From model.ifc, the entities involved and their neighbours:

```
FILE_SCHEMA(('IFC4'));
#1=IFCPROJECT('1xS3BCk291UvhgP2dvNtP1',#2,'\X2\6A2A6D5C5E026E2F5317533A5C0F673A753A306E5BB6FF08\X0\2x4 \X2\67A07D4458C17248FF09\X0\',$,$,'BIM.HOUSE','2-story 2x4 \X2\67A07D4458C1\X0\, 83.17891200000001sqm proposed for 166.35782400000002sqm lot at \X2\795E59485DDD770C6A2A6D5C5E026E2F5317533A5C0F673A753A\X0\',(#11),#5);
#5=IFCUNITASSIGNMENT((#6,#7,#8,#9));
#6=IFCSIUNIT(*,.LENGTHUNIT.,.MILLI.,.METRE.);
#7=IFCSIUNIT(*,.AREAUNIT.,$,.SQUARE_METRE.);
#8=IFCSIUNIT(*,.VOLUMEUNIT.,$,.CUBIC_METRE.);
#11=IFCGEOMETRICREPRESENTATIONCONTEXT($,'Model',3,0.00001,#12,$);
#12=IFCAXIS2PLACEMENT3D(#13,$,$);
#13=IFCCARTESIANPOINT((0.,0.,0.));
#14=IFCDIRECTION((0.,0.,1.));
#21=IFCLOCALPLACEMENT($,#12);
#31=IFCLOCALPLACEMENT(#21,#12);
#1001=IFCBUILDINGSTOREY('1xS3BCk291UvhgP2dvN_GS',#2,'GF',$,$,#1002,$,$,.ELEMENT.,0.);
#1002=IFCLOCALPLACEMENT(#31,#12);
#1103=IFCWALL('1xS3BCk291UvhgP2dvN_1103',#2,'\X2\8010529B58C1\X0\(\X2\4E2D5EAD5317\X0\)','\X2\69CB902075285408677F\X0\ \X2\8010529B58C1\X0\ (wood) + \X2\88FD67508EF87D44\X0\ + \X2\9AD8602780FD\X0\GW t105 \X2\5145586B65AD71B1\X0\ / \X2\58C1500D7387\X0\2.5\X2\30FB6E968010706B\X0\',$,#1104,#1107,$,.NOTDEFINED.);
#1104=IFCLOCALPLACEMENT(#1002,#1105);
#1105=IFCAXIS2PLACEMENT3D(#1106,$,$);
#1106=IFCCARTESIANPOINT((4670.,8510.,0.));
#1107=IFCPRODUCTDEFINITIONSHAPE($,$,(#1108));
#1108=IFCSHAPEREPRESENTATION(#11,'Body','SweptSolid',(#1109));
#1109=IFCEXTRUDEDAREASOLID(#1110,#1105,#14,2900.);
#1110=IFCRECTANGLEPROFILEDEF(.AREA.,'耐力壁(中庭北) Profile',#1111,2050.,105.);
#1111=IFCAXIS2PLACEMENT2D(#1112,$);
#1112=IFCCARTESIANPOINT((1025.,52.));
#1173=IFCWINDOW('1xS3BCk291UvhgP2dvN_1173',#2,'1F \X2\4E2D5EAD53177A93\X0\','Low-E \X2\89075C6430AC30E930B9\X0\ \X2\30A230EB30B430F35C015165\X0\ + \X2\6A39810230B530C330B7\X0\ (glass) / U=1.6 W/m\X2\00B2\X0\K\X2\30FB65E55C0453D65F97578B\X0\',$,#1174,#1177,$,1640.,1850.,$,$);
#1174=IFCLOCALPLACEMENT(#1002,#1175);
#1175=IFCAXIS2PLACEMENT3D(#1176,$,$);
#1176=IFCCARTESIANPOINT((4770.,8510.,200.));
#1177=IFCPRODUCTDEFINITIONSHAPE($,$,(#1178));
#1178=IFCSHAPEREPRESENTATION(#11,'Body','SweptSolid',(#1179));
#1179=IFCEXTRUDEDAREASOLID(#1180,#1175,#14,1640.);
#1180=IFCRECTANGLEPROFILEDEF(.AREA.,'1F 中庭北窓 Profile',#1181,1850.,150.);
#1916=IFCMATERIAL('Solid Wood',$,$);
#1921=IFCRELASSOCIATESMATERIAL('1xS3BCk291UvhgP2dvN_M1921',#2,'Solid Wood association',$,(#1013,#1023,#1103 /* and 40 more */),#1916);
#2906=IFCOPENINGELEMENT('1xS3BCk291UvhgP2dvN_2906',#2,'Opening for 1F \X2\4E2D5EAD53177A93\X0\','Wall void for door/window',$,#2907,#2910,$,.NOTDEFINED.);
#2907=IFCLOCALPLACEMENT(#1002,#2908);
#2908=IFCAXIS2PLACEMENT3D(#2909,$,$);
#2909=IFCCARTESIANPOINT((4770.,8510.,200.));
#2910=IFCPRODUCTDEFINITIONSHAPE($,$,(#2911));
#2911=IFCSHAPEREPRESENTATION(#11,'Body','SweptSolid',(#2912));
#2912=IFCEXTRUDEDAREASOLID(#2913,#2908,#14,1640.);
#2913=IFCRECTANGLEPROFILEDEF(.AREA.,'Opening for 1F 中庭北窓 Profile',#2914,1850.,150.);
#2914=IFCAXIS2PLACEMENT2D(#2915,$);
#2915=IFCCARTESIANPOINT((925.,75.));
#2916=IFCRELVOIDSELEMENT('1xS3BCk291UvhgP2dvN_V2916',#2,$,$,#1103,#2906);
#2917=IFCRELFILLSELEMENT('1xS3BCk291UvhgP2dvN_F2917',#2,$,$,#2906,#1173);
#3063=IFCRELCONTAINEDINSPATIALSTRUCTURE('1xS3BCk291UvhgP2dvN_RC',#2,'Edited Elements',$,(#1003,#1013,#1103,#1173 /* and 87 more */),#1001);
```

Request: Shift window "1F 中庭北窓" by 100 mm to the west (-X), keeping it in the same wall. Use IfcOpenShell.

```python
import ifcopenshell
import ifcopenshell.api.geometry
import ifcopenshell.util.placement
import ifcopenshell.util.unit

model = ifcopenshell.open("model.ifc")
unit_scale = ifcopenshell.util.unit.calculate_unit_scale(model)

window = model.by_guid("1xS3BCk291UvhgP2dvN_1173")
opening = window.FillsVoids[0].RelatingOpeningElement
wall = opening.VoidsElements[0].RelatingBuildingElement

wall_matrix = ifcopenshell.util.placement.get_local_placement(wall.ObjectPlacement)
shift = wall_matrix[:3, 0] * -0.1 / unit_scale
before = ifcopenshell.util.placement.get_local_placement(window.ObjectPlacement)[:3, 3].copy()

# The window is not placed relative to its opening, so move both.
for product in (opening, window):
    matrix = ifcopenshell.util.placement.get_local_placement(product.ObjectPlacement)
    matrix[:3, 3] += shift
    ifcopenshell.api.geometry.edit_object_placement(model, product=product, matrix=matrix, is_si=False)

after = ifcopenshell.util.placement.get_local_placement(window.ObjectPlacement)[:3, 3]
print("window moved by", (after - before).round(3) + 0.0)

model.write("model-out.ifc")
```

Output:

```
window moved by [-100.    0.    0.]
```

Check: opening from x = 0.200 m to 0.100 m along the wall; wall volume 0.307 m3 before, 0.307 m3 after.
